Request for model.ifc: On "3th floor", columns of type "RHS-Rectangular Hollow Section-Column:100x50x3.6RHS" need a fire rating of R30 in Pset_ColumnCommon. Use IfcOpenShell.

First a look at what the model holds.

```python
import ifcopenshell
import ifcopenshell.util.element

model = ifcopenshell.open("model.ifc")
print(model.schema)
storey = next(s for s in model.by_type("IfcBuildingStorey") if s.Name == "3th floor")
columns = [e for e in ifcopenshell.util.element.get_decomposition(storey) if e.is_a("IfcColumn")]
seen = {}
for e in columns:
    element_type = ifcopenshell.util.element.get_type(e)
    key = (element_type.Name if element_type != e and element_type else None, ifcopenshell.util.element.get_pset(e, "Pset_ColumnCommon", "FireRating"))
    seen[key] = seen.get(key, 0) + 1
for (name, value), count in sorted(seen.items(), key=str):
    print(count, "x", name, "|", value)
```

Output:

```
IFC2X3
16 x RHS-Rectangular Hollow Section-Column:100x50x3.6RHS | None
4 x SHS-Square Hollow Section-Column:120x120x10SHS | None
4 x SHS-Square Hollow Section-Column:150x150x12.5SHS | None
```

```python
import ifcopenshell
import ifcopenshell.api.pset
import ifcopenshell.util.element

model = ifcopenshell.open("model.ifc")

storey = next(s for s in model.by_type("IfcBuildingStorey") if s.Name == "3th floor")
columns = [e for e in ifcopenshell.util.element.get_decomposition(storey) if e.is_a("IfcColumn")]

count = 0
for e in columns:
    element_type = ifcopenshell.util.element.get_type(e)
    if element_type in (None, e) or element_type.Name != "RHS-Rectangular Hollow Section-Column:100x50x3.6RHS":
        continue
    # add_pset returns the element's existing set when there is one.
    pset = ifcopenshell.api.pset.add_pset(model, product=e, name="Pset_ColumnCommon")
    ifcopenshell.api.pset.edit_pset(model, pset=pset, properties={"FireRating": "R30"})
    count += 1

print(count, "columns updated")

model.write("model_v2.ifc")
```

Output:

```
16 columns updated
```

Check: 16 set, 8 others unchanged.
